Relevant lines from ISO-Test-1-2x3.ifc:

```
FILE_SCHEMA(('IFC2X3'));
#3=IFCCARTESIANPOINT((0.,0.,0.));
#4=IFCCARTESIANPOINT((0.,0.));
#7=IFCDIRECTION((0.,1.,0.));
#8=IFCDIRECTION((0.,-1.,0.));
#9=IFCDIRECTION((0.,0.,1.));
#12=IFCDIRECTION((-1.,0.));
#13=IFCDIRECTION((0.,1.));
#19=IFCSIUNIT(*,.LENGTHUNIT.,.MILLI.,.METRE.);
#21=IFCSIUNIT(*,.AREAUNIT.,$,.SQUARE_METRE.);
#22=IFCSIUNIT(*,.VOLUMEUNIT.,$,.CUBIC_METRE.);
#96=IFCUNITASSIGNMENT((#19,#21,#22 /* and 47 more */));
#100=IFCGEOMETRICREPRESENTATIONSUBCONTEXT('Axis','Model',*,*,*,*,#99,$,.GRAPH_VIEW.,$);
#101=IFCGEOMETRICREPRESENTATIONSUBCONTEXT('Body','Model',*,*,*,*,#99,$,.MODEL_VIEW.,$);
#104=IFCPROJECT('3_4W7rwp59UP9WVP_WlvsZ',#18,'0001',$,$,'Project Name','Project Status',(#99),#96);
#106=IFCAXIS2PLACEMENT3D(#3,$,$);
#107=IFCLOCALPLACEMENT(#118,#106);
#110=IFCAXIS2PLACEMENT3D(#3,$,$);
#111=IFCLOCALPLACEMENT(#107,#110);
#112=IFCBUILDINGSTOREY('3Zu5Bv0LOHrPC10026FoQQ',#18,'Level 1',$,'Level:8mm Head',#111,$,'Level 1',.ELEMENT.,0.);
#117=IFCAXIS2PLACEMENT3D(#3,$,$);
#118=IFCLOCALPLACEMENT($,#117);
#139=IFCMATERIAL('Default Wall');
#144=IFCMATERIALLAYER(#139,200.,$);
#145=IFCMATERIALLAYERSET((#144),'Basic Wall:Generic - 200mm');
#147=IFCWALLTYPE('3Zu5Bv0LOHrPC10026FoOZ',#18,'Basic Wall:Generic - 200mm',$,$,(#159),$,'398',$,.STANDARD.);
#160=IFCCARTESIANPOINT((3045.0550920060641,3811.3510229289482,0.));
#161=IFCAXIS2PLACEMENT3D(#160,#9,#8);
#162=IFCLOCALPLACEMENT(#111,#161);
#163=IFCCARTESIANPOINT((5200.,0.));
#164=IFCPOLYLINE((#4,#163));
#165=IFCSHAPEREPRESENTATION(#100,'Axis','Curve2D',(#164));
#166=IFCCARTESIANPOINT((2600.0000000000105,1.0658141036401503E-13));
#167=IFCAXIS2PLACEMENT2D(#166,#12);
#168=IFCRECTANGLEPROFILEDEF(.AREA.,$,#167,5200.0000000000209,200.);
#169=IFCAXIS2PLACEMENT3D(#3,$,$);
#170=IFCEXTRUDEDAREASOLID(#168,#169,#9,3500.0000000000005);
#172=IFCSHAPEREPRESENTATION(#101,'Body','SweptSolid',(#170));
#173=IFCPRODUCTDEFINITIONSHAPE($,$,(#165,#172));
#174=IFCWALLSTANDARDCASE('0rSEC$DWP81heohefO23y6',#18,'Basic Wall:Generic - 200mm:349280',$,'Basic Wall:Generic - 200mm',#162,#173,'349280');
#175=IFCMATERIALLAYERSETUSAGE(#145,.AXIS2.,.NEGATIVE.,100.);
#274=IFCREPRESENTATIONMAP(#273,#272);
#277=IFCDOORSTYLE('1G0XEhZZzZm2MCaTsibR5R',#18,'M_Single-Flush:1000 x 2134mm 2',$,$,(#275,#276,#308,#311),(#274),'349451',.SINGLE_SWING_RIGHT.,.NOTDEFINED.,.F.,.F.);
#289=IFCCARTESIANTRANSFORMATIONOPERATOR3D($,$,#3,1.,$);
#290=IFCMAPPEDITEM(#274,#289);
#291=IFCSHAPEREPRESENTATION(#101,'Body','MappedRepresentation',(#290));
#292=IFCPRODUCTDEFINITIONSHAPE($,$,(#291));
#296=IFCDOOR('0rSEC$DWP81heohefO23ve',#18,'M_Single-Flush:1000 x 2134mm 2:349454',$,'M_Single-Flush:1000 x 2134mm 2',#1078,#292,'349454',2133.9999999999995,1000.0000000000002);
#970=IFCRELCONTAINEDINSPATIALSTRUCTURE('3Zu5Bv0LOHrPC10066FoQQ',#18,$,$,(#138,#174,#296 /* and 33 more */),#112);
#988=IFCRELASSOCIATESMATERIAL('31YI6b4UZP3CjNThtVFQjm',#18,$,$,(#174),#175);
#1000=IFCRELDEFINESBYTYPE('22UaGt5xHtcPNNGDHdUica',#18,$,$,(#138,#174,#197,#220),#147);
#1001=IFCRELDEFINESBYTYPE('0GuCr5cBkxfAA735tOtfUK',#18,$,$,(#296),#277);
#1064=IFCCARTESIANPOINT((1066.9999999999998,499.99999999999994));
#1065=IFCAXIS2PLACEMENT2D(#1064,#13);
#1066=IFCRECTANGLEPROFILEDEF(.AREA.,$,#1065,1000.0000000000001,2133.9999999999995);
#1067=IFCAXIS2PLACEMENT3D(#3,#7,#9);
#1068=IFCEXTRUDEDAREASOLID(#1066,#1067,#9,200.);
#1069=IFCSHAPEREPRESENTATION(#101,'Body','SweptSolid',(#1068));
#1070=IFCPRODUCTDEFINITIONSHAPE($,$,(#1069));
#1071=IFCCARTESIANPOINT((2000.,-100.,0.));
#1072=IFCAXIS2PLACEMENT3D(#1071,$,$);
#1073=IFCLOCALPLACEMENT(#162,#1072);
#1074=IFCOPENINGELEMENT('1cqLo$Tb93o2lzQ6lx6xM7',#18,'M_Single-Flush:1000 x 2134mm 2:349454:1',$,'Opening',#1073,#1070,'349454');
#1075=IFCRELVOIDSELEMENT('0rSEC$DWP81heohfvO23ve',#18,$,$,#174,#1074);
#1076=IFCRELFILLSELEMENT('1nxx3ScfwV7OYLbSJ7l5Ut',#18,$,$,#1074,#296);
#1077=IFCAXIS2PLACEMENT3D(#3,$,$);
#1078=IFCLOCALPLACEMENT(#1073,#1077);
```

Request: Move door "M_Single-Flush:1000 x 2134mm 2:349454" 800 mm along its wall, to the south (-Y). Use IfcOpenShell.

```python
import ifcopenshell
import ifcopenshell.api.geometry
import ifcopenshell.util.placement

model = ifcopenshell.open("ISO-Test-1-2x3.ifc")

door = model.by_guid("0rSEC$DWP81heohefO23ve")
opening = door.FillsVoids[0].RelatingOpeningElement
wall = opening.VoidsElements[0].RelatingBuildingElement

wall_matrix = ifcopenshell.util.placement.get_local_placement(wall.ObjectPlacement)
shift = wall_matrix[:3, 0] * 800.0
before = ifcopenshell.util.placement.get_local_placement(door.ObjectPlacement)[:3, 3].copy()

# The door is placed relative to its opening, so it follows when the opening moves.
matrix = ifcopenshell.util.placement.get_local_placement(opening.ObjectPlacement)
matrix[:3, 3] += shift
ifcopenshell.api.geometry.edit_object_placement(
    model, product=opening, matrix=matrix, is_si=False, should_transform_children=True
)

after = ifcopenshell.util.placement.get_local_placement(door.ObjectPlacement)[:3, 3]
print("door moved by", (after - before).round(3) + 0.0)

model.write("ISO-Test-1-2x3_v2.ifc")
```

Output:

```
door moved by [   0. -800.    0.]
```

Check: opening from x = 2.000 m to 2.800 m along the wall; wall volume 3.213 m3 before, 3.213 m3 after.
